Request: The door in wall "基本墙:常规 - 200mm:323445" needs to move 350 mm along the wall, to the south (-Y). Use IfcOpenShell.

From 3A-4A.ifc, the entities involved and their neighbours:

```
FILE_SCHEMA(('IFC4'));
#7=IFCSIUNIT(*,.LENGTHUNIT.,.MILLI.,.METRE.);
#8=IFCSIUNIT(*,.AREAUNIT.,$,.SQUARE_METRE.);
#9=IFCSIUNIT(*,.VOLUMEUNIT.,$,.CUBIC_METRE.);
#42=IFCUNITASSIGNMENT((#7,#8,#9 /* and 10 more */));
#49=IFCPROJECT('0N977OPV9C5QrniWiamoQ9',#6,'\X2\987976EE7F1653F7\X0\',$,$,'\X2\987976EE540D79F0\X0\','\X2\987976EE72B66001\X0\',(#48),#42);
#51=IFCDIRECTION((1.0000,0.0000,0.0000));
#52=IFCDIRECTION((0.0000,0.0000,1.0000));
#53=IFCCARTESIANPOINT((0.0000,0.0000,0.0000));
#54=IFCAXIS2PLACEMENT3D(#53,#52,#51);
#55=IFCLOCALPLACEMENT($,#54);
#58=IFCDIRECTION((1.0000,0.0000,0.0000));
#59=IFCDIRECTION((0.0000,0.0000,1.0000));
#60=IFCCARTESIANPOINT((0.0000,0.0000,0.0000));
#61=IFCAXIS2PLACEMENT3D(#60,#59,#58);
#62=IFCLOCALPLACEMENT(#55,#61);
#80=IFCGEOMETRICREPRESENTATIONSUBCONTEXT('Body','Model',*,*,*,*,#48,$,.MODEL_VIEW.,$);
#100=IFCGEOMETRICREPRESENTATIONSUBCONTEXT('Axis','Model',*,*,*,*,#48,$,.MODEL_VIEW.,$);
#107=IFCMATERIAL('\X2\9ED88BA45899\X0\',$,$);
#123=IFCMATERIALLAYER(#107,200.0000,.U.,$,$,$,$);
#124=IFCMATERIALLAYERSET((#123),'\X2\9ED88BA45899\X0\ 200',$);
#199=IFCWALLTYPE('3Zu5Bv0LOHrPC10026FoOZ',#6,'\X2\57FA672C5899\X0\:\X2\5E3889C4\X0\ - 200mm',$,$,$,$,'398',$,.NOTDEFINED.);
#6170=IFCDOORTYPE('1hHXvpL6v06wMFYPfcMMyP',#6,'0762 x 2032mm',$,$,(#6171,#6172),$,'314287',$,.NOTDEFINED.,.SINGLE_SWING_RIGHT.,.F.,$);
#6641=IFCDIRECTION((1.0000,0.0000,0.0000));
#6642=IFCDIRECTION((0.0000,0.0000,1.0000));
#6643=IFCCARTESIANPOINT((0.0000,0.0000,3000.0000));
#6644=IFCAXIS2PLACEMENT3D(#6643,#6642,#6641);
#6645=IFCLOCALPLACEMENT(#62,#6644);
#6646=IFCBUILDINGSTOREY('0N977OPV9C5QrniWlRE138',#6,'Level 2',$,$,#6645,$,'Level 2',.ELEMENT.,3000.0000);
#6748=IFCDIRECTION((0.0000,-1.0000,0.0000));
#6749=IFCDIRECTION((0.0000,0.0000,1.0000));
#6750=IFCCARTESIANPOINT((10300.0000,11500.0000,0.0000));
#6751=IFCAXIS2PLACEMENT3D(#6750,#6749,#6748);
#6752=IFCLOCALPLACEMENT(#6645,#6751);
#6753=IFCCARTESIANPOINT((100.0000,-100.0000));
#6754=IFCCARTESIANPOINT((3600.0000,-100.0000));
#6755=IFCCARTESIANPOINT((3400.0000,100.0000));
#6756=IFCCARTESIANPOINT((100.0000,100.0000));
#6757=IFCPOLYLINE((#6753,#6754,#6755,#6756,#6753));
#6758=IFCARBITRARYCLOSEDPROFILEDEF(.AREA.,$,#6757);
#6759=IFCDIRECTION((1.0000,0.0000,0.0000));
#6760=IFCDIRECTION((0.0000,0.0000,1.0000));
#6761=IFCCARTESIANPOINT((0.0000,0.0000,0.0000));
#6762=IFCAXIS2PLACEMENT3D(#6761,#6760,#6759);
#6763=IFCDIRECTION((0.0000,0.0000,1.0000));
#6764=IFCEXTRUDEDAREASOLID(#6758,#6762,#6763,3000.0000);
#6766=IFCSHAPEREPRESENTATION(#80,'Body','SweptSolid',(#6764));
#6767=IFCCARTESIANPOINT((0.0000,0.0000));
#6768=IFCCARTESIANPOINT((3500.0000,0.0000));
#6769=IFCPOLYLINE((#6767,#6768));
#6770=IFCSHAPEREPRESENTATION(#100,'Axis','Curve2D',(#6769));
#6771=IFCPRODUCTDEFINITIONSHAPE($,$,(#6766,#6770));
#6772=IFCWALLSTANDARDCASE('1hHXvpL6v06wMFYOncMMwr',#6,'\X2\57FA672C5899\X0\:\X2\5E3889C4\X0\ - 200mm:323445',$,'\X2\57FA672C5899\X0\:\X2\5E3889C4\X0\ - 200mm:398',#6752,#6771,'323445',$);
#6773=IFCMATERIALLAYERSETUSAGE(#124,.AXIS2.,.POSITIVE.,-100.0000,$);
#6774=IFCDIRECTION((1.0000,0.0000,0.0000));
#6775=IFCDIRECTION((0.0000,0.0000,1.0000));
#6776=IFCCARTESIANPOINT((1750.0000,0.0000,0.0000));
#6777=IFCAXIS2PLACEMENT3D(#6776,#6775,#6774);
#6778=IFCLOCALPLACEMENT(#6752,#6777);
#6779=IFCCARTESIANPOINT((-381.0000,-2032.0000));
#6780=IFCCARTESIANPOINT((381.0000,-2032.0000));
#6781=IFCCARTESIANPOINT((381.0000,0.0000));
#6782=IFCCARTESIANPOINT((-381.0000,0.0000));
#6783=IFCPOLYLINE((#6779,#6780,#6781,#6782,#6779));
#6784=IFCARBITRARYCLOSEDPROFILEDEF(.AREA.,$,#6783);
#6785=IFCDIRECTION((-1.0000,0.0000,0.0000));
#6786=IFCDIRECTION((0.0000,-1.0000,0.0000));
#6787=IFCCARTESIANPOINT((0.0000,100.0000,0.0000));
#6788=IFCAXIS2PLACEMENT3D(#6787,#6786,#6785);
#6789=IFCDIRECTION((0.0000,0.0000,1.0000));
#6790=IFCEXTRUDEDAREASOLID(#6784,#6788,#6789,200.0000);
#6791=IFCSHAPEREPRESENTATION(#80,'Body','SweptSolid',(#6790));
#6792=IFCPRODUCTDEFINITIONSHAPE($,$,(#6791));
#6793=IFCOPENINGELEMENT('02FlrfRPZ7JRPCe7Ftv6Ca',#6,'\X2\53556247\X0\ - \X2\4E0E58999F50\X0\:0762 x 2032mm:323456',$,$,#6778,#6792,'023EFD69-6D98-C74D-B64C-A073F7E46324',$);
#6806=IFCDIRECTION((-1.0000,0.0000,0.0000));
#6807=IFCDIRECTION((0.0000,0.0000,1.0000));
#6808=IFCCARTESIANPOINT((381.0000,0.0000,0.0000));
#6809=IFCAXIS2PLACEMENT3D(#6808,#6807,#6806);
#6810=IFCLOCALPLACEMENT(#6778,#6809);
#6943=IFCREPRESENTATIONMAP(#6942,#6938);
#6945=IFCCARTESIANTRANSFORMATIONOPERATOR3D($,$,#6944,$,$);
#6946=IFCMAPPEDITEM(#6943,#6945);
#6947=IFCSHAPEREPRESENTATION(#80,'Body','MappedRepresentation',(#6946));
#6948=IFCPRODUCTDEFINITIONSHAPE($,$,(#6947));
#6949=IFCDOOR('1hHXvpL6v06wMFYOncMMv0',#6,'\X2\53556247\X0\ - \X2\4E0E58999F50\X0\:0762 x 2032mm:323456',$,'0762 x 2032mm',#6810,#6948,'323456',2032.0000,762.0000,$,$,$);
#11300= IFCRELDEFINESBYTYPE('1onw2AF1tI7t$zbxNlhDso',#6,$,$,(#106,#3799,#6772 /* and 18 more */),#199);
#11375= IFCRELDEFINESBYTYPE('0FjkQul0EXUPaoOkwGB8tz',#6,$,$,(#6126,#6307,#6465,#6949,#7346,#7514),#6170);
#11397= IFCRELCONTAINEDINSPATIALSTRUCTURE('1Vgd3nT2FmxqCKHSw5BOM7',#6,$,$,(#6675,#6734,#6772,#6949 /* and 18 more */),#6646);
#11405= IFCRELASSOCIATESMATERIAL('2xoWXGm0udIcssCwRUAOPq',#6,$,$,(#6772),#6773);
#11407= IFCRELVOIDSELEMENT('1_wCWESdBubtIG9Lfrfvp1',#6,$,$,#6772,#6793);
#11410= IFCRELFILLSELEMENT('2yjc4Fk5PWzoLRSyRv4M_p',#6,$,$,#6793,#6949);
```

```python
import ifcopenshell
import ifcopenshell.api.geometry
import ifcopenshell.util.placement

model = ifcopenshell.open("3A-4A.ifc")

door = model.by_id(6949)
opening = door.FillsVoids[0].RelatingOpeningElement
wall = opening.VoidsElements[0].RelatingBuildingElement

wall_matrix = ifcopenshell.util.placement.get_local_placement(wall.ObjectPlacement)
shift = wall_matrix[:3, 0] * 350.0
before = ifcopenshell.util.placement.get_local_placement(door.ObjectPlacement)[:3, 3].copy()

# The door is placed relative to its opening, so it follows when the opening moves.
matrix = ifcopenshell.util.placement.get_local_placement(opening.ObjectPlacement)
matrix[:3, 3] += shift
ifcopenshell.api.geometry.edit_object_placement(
    model, product=opening, matrix=matrix, is_si=False, should_transform_children=True
)

after = ifcopenshell.util.placement.get_local_placement(door.ObjectPlacement)[:3, 3]
print("door moved by", (after - before).round(3) + 0.0)

model.write("3A-4A-out.ifc")
```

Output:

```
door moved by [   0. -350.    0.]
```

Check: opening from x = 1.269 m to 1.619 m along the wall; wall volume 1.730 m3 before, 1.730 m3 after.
